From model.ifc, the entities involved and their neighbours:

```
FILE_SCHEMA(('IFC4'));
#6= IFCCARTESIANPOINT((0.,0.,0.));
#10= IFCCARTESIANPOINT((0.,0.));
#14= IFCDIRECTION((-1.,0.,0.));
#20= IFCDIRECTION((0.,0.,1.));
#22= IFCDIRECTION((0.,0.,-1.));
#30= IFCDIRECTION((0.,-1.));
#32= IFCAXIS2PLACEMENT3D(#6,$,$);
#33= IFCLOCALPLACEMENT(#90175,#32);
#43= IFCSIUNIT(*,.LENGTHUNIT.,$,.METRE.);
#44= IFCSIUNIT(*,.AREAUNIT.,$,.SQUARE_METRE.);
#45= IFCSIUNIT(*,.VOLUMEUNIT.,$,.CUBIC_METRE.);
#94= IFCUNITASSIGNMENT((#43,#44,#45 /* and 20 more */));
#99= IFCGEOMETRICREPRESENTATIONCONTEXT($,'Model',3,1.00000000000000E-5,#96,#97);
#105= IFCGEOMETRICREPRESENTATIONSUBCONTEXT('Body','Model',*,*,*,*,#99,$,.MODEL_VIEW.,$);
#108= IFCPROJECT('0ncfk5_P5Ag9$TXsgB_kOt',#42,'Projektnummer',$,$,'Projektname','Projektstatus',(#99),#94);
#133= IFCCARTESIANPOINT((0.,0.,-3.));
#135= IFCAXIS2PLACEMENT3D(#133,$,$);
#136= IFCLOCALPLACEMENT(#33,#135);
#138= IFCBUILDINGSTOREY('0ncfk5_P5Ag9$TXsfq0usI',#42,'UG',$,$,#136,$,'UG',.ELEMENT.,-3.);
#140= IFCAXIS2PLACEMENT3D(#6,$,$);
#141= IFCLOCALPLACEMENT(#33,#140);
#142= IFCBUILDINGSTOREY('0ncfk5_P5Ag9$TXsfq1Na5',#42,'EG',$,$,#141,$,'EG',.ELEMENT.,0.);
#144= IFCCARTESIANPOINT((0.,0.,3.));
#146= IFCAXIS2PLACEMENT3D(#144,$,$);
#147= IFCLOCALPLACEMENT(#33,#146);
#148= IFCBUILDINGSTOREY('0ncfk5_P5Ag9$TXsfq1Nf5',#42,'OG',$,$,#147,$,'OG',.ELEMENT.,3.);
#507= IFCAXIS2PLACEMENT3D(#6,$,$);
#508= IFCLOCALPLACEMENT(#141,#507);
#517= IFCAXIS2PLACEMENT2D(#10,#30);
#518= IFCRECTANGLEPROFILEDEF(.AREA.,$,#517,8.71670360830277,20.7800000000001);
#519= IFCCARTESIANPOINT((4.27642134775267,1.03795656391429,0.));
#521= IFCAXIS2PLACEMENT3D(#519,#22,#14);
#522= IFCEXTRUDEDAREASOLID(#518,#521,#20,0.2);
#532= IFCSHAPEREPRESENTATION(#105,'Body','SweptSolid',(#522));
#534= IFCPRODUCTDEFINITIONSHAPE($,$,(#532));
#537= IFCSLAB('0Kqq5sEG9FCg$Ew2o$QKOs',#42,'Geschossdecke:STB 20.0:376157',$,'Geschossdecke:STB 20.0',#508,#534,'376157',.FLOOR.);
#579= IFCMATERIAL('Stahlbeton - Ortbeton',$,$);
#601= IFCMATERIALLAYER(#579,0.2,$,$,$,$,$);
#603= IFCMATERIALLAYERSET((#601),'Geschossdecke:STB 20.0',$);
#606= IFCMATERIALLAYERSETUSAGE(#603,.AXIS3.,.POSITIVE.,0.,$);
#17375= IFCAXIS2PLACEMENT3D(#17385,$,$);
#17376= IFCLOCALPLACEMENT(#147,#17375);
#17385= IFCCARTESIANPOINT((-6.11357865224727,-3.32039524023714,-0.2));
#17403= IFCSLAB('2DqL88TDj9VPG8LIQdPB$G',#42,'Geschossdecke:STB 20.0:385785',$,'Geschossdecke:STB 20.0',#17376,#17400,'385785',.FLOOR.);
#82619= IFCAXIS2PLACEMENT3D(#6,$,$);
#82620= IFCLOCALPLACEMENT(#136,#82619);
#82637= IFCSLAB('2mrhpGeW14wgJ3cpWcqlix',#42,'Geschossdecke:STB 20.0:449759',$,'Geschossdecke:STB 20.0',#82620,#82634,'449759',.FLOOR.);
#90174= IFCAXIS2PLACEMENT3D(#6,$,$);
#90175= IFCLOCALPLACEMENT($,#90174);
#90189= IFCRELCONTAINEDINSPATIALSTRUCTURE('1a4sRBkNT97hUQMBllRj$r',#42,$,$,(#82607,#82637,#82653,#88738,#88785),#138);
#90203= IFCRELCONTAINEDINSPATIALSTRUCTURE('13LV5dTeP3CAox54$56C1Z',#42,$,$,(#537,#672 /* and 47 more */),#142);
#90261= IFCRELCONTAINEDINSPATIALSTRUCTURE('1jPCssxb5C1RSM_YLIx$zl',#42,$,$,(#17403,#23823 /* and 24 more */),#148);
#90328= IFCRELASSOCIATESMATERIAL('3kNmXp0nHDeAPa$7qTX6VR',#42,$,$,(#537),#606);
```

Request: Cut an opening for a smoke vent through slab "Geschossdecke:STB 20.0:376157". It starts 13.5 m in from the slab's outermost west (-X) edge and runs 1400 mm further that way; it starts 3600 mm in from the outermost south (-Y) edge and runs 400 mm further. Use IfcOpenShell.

```python
import numpy as np
import ifcopenshell
import ifcopenshell.api.feature
import ifcopenshell.api.geometry
import ifcopenshell.api.root
import ifcopenshell.geom
import ifcopenshell.util.placement
import ifcopenshell.util.representation
import ifcopenshell.util.shape
import ifcopenshell.util.unit

model = ifcopenshell.open("model.ifc")
unit_scale = ifcopenshell.util.unit.calculate_unit_scale(model)
settings = ifcopenshell.geom.settings()


def volume(element):
    """Net volume in cubic metres, openings subtracted."""
    shape = ifcopenshell.geom.create_shape(settings, element)
    return ifcopenshell.util.shape.get_volume(shape.geometry)


slab = model.by_guid("0Kqq5sEG9FCg$Ew2o$QKOs")
before = volume(slab)

# Extent in the slab's own axes, in metres. The edges named are its -X and -Y sides.
slab_shape = ifcopenshell.geom.create_shape(settings, slab)
vertices = ifcopenshell.util.shape.get_vertices(slab_shape.geometry)
x_min, y_min, bottom = vertices.min(axis=0)
top = vertices[:, 2].max()

opening = ifcopenshell.api.root.create_entity(model, ifc_class="IfcOpeningElement", name="Smoke vent opening", predefined_type="OPENING")
context = ifcopenshell.util.representation.get_context(model, "Model", "Body", "MODEL_VIEW")
width, depth = 1.4, 0.4
outline = [(0.0, 0.0), (width, 0.0), (width, depth), (0.0, depth), (0.0, 0.0)]
# Overshoot both faces by 50 mm so the cut is clean.
shape = ifcopenshell.api.geometry.add_slab_representation(
    model, context=context, depth=top - bottom + 0.1, polyline=outline
)
ifcopenshell.api.geometry.assign_representation(model, product=opening, representation=shape)

matrix = ifcopenshell.util.placement.get_local_placement(slab.ObjectPlacement)
matrix[:, 3] = matrix @ np.append(np.array([x_min + 13.5, y_min + 3.6, bottom - 0.05]) / unit_scale, 1.0)
ifcopenshell.api.geometry.edit_object_placement(model, product=opening, matrix=matrix, is_si=False)
ifcopenshell.api.feature.add_feature(model, feature=opening, element=slab)

after = volume(slab)

print(f"slab volume {before:.3f} -> {after:.3f} m3")

model.write("model_v2.ifc")
```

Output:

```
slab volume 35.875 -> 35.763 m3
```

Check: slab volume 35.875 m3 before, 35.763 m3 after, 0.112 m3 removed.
